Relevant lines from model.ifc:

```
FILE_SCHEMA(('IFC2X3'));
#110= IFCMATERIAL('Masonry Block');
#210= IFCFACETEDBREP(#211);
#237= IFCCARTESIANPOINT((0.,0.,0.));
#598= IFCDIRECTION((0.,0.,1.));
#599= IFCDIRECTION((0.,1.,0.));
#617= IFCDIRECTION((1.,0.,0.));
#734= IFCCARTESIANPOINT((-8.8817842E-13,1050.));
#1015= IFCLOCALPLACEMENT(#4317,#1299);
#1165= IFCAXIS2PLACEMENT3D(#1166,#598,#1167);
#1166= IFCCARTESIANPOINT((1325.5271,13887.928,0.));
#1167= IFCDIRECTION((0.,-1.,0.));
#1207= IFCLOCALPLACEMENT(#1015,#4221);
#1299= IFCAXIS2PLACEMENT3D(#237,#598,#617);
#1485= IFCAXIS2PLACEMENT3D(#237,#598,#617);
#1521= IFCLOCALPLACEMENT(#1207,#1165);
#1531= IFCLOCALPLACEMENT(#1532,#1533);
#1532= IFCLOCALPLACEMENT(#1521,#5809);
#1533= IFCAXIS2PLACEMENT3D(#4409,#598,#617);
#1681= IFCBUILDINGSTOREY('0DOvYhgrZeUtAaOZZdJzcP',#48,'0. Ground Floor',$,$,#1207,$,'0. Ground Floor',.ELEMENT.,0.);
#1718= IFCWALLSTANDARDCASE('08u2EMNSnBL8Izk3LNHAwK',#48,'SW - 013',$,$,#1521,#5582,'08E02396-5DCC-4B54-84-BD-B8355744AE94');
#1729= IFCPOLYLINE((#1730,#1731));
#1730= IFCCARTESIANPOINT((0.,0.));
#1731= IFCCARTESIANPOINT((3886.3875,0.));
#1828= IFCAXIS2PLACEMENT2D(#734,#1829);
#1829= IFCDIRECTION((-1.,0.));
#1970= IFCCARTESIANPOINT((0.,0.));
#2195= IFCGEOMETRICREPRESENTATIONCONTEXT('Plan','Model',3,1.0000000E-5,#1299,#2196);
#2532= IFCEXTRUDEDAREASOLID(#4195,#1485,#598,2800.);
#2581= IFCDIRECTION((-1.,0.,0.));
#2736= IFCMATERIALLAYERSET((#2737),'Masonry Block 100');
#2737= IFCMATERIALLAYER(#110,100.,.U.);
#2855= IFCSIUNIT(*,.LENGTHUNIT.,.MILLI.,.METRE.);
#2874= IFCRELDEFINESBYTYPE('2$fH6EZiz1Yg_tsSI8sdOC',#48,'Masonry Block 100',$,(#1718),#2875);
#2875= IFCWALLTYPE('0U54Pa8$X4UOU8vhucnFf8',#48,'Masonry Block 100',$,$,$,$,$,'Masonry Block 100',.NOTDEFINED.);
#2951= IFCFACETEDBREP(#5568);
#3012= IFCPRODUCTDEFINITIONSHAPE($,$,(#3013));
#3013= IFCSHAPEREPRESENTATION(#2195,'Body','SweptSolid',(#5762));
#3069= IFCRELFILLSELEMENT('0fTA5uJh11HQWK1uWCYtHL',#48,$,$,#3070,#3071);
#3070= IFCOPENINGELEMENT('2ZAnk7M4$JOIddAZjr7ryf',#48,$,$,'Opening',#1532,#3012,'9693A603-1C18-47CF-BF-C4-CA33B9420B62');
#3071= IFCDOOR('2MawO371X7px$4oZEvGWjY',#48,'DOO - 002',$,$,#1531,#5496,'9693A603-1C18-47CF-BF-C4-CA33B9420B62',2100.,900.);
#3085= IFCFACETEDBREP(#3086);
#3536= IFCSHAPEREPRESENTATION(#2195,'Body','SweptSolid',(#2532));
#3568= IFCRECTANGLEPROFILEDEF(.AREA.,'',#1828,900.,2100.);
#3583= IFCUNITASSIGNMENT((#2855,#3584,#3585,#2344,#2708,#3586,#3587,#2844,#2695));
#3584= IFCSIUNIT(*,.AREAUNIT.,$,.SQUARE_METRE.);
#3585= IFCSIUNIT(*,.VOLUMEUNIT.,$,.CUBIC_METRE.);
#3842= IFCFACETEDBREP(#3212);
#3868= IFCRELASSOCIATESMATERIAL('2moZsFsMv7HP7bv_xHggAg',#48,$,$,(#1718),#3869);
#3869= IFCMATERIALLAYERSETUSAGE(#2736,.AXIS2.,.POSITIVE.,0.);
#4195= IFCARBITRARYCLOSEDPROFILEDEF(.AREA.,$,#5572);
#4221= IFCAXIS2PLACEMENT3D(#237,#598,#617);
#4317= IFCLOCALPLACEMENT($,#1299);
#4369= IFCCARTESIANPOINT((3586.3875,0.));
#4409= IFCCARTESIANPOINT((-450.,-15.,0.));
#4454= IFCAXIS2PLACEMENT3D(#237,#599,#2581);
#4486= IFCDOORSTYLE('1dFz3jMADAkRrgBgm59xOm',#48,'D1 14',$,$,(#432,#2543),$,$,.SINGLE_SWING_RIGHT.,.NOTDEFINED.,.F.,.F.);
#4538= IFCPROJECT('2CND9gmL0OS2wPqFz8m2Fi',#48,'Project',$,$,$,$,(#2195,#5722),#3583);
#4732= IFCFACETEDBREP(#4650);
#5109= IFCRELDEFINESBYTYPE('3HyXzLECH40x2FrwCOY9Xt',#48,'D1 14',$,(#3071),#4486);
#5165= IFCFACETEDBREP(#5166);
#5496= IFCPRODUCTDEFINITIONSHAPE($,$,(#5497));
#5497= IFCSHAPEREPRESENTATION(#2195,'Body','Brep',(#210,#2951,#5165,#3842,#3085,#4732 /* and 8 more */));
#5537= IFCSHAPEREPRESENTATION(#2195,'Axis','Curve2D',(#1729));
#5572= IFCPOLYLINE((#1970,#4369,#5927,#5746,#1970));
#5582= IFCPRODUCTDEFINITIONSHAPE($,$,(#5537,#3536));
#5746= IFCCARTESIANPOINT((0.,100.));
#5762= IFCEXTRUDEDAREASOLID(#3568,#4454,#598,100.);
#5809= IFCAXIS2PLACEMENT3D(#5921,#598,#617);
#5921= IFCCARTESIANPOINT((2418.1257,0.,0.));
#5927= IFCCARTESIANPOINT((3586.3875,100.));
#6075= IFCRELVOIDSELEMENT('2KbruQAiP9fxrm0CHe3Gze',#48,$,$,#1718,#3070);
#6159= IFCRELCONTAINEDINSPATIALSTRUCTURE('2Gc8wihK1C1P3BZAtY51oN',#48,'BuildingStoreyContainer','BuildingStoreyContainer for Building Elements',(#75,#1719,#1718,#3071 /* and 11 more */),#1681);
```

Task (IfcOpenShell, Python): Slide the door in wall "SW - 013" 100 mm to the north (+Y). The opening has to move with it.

```python
import ifcopenshell
import ifcopenshell.api.geometry
import ifcopenshell.util.placement

model = ifcopenshell.open("model.ifc")

door = model.by_guid("2MawO371X7px$4oZEvGWjY")
opening = door.FillsVoids[0].RelatingOpeningElement
wall = opening.VoidsElements[0].RelatingBuildingElement

wall_matrix = ifcopenshell.util.placement.get_local_placement(wall.ObjectPlacement)
shift = wall_matrix[:3, 0] * -100.0
before = ifcopenshell.util.placement.get_local_placement(door.ObjectPlacement)[:3, 3].copy()

# The door is placed relative to its opening, so it follows when the opening moves.
matrix = ifcopenshell.util.placement.get_local_placement(opening.ObjectPlacement)
matrix[:3, 3] += shift
ifcopenshell.api.geometry.edit_object_placement(
    model, product=opening, matrix=matrix, is_si=False, should_transform_children=True
)

after = ifcopenshell.util.placement.get_local_placement(door.ObjectPlacement)[:3, 3]
print("door moved by", (after - before).round(3) + 0.0)

model.write("model-out.ifc")
```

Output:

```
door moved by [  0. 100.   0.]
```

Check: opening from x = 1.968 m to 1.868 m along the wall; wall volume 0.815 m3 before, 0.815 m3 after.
